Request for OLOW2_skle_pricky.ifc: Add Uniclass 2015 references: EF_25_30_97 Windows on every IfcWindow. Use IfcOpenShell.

First a look at what the model holds.

```python
import ifcopenshell

model = ifcopenshell.open("OLOW2_skle_pricky.ifc")
print(model.schema)
print("classifications:", [c.Name for c in model.by_type("IfcClassification")])
for ifc_class in ("IfcDoor", "IfcRoof", "IfcStair", "IfcWall", "IfcWindow"):
    print(ifc_class, len(model.by_type(ifc_class)))
```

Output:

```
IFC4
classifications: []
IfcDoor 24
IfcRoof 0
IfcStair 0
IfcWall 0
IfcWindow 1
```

```python
import ifcopenshell
import ifcopenshell.api.classification

model = ifcopenshell.open("OLOW2_skle_pricky.ifc")

system = ifcopenshell.api.classification.add_classification(model, classification="Uniclass 2015")

codes = {
    "IfcWindow": ("EF_25_30_97", "Windows"),
}
for ifc_class, (code, name) in codes.items():
    products = model.by_type(ifc_class)
    ifcopenshell.api.classification.add_reference(
        model, products=products, classification=system, identification=code, name=name
    )
    print(code, len(products))

model.write("OLOW2_skle_pricky_updated.ifc")
```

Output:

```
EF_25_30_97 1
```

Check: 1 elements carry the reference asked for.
